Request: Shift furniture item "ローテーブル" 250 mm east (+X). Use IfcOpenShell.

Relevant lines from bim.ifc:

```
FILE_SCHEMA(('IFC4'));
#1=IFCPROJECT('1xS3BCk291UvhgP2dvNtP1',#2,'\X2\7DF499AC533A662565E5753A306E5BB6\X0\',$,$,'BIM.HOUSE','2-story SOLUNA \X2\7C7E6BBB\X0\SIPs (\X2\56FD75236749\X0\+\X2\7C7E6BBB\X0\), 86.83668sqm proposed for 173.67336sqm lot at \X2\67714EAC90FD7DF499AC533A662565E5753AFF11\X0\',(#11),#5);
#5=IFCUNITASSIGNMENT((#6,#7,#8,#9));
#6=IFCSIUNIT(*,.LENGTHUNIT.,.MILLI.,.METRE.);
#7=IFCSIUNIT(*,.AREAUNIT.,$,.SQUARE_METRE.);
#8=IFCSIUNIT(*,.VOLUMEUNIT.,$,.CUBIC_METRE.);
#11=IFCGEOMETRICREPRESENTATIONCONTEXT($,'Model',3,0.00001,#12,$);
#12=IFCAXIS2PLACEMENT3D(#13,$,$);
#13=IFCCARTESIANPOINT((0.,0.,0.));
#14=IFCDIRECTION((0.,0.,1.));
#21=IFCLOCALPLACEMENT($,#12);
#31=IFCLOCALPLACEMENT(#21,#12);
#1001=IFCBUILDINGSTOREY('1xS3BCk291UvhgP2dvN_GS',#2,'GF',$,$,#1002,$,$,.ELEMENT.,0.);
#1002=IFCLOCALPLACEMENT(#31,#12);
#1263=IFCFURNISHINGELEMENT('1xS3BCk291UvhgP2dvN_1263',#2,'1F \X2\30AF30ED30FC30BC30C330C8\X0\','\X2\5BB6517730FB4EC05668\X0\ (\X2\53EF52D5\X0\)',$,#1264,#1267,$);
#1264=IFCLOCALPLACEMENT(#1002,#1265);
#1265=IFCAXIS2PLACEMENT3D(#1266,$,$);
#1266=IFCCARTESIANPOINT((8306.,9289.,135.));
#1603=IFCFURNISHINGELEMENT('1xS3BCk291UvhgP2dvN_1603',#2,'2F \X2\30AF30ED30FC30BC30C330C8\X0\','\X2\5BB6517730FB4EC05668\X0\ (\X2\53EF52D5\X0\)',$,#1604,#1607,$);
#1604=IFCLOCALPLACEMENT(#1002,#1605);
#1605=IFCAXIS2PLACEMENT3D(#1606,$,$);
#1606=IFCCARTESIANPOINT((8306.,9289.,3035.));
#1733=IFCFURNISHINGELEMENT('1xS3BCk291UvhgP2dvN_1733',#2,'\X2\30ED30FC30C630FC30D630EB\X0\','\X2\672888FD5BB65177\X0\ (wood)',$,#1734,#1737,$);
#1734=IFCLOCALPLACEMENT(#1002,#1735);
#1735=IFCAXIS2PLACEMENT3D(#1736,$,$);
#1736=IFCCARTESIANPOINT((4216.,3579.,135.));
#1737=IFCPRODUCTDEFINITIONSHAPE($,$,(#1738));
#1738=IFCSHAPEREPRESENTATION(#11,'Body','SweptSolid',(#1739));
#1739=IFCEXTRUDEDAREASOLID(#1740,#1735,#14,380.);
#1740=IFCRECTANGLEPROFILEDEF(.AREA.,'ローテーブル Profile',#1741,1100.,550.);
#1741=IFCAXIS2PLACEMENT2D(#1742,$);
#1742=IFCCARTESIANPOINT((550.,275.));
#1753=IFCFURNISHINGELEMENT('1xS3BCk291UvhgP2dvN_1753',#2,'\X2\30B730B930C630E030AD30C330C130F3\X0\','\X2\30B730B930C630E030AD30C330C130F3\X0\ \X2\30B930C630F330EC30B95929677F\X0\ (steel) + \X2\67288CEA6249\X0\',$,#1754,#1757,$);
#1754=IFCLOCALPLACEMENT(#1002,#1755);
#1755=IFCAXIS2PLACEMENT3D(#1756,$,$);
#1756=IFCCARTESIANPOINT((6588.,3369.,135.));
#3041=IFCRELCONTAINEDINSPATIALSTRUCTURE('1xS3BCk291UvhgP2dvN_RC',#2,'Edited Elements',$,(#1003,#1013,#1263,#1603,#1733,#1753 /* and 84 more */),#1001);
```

```python
import ifcopenshell
import ifcopenshell.api.geometry
import ifcopenshell.util.placement

model = ifcopenshell.open("bim.ifc")

item = model.by_guid("1xS3BCk291UvhgP2dvN_1733")
matrix = ifcopenshell.util.placement.get_local_placement(item.ObjectPlacement)
matrix[0, 3] += 250.0
ifcopenshell.api.geometry.edit_object_placement(model, product=item, matrix=matrix, is_si=False)

print(ifcopenshell.util.placement.get_local_placement(item.ObjectPlacement).round(3) + 0.0)

model.write("bim-out.ifc")
```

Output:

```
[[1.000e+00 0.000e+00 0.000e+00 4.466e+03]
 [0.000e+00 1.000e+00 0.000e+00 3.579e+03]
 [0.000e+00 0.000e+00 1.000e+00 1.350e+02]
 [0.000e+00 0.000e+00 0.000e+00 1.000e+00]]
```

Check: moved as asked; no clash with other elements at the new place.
